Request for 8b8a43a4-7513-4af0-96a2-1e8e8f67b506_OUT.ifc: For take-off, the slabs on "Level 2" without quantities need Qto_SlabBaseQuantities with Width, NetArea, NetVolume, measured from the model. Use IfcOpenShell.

First a look at what the model holds.

```python
import ifcopenshell
import ifcopenshell.util.element
import ifcopenshell.util.unit

model = ifcopenshell.open("8b8a43a4-7513-4af0-96a2-1e8e8f67b506_OUT.ifc")
print(model.schema)
for unit_type in ("LENGTHUNIT", "AREAUNIT", "VOLUMEUNIT"):
    print(unit_type, ifcopenshell.util.unit.calculate_unit_scale(model, unit_type))
storey = next(s for s in model.by_type("IfcBuildingStorey") if s.Name == "Level 2")
slabs = [e for e in ifcopenshell.util.element.get_decomposition(storey) if e.is_a("IfcSlab")]
for e in sorted(slabs, key=lambda e: e.id()):
    print(e.id(), e.is_a(), e.Name, list(ifcopenshell.util.element.get_psets(e, qtos_only=True)), sep=" | ")
```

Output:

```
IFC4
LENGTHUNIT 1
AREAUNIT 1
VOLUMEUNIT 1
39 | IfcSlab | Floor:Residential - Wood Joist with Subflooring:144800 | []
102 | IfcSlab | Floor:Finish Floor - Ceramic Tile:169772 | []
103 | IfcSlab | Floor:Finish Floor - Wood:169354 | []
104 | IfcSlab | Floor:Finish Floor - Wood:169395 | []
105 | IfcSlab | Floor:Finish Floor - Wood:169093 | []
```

```python
import ifcopenshell
import ifcopenshell.api.pset
import ifcopenshell.geom
import ifcopenshell.util.element
import ifcopenshell.util.shape
import ifcopenshell.util.unit

model = ifcopenshell.open("8b8a43a4-7513-4af0-96a2-1e8e8f67b506_OUT.ifc")
unit_scale = ifcopenshell.util.unit.calculate_unit_scale(model)
area_scale = ifcopenshell.util.unit.calculate_unit_scale(model, "AREAUNIT")
volume_scale = ifcopenshell.util.unit.calculate_unit_scale(model, "VOLUMEUNIT")
settings = ifcopenshell.geom.settings()

storey = next(s for s in model.by_type("IfcBuildingStorey") if s.Name == "Level 2")
slabs = [e for e in ifcopenshell.util.element.get_decomposition(storey) if e.is_a("IfcSlab")]

for e in sorted(slabs, key=lambda e: e.id()):
    if ifcopenshell.util.element.get_psets(e, qtos_only=True, should_inherit=False):
        continue
    # Geometry comes back in metres, in the element's own axes.
    shape = ifcopenshell.geom.create_shape(settings, e)
    values = {
        "Width": ifcopenshell.util.shape.get_z(shape.geometry) / unit_scale,
        "NetArea": ifcopenshell.util.shape.get_footprint_area(shape.geometry) / area_scale,
        "NetVolume": ifcopenshell.util.shape.get_volume(shape.geometry) / volume_scale,
    }
    qto = ifcopenshell.api.pset.add_qto(model, product=e, name="Qto_SlabBaseQuantities")
    ifcopenshell.api.pset.edit_qto(model, qto=qto, properties=values)
    print(e.id(), {k: round(v, 3) for k, v in values.items()})

model.write("8b8a43a4-7513-4af0-96a2-1e8e8f67b506_OUT_edited.ifc")
```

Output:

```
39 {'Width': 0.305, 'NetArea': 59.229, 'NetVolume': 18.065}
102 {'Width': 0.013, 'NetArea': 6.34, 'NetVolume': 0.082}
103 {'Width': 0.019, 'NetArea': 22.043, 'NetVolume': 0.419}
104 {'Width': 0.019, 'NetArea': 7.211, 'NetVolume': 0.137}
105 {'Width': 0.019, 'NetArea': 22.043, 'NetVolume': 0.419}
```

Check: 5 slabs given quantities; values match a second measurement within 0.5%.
